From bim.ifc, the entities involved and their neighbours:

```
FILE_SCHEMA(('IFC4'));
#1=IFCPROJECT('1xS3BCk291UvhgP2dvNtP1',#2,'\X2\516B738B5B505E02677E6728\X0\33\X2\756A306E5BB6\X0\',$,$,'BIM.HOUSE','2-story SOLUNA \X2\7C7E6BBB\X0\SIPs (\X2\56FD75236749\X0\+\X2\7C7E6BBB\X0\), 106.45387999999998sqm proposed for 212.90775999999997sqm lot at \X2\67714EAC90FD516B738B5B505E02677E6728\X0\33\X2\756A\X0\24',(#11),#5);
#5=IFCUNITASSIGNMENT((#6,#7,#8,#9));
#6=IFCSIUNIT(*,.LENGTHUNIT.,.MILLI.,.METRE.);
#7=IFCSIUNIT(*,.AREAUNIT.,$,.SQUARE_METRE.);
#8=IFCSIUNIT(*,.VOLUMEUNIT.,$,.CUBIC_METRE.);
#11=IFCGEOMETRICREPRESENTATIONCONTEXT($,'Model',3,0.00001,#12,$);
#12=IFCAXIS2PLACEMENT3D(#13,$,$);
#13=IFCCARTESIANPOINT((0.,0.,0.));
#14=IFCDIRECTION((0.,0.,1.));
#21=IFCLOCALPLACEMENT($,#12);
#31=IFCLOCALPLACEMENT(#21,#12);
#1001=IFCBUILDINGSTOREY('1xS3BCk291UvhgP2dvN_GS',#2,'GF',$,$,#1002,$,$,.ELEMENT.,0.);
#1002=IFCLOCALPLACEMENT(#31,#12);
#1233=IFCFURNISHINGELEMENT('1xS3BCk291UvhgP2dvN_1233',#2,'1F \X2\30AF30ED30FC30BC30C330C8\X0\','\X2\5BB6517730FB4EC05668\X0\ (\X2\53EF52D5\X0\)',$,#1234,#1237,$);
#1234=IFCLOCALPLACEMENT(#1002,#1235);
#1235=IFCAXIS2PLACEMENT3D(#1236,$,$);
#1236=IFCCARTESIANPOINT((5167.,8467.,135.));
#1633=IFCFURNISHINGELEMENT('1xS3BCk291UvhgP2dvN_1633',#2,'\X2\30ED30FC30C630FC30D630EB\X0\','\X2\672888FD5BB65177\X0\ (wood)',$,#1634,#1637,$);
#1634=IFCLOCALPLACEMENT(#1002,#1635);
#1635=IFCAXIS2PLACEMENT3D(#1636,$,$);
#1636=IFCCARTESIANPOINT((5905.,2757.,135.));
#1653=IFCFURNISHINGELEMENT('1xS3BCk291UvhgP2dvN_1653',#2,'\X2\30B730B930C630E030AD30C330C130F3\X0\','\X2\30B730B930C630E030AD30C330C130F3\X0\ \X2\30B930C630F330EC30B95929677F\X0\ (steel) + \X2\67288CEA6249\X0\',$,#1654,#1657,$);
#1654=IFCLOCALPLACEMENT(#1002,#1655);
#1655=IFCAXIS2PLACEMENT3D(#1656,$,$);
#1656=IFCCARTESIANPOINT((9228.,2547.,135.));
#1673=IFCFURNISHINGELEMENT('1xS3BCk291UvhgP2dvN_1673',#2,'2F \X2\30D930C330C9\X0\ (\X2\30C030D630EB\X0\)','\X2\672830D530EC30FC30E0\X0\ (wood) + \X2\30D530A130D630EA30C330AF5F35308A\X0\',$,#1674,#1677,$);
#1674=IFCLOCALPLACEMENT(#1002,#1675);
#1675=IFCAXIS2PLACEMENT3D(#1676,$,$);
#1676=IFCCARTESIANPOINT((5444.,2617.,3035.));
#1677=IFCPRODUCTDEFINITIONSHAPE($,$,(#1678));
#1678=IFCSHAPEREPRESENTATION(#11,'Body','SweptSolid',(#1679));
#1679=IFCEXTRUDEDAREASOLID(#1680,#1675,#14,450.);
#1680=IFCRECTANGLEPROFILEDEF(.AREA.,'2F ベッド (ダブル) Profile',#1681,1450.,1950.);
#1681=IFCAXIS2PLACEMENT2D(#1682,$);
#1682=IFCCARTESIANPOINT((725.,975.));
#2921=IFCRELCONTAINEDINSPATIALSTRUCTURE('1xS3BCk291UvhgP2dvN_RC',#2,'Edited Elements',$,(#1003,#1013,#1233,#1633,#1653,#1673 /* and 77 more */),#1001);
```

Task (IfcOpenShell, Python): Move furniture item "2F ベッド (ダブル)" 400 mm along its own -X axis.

```python
import ifcopenshell
import ifcopenshell.api.geometry
import ifcopenshell.util.placement
import ifcopenshell.util.unit

model = ifcopenshell.open("bim.ifc")
unit_scale = ifcopenshell.util.unit.calculate_unit_scale(model)

item = model.by_id(1673)
matrix = ifcopenshell.util.placement.get_local_placement(item.ObjectPlacement)
matrix[:3, 3] -= matrix[:3, 0] * 0.4 / unit_scale
ifcopenshell.api.geometry.edit_object_placement(model, product=item, matrix=matrix, is_si=False)

print(ifcopenshell.util.placement.get_local_placement(item.ObjectPlacement).round(3) + 0.0)

model.write("bim_v2.ifc")
```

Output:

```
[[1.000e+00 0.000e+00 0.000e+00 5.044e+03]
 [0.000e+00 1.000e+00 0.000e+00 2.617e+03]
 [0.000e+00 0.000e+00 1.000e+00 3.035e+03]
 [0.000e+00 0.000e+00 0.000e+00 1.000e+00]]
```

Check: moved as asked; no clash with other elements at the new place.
